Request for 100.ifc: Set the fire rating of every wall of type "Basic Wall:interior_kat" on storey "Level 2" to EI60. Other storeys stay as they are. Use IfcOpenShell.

First a look at what the model holds.

```python
import ifcopenshell
import ifcopenshell.util.element

model = ifcopenshell.open("100.ifc")
print(model.schema)
storey = next(s for s in model.by_type("IfcBuildingStorey") if s.Name == "Level 2")
walls = [e for e in ifcopenshell.util.element.get_decomposition(storey) if e.is_a("IfcWall")]
seen = {}
for e in walls:
    element_type = ifcopenshell.util.element.get_type(e)
    key = (element_type.Name if element_type != e and element_type else None, ifcopenshell.util.element.get_pset(e, "Pset_WallCommon", "FireRating"))
    seen[key] = seen.get(key, 0) + 1
for (name, value), count in sorted(seen.items(), key=str):
    print(count, "x", name, "|", value)
```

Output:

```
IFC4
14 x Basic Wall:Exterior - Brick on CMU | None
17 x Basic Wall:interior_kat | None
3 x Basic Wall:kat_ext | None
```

```python
import ifcopenshell
import ifcopenshell.api.pset
import ifcopenshell.util.element

model = ifcopenshell.open("100.ifc")

storey = next(s for s in model.by_type("IfcBuildingStorey") if s.Name == "Level 2")
walls = [e for e in ifcopenshell.util.element.get_decomposition(storey) if e.is_a("IfcWall")]

count = 0
for e in walls:
    element_type = ifcopenshell.util.element.get_type(e)
    if element_type in (None, e) or element_type.Name != "Basic Wall:interior_kat":
        continue
    # add_pset returns the element's existing set when there is one.
    pset = ifcopenshell.api.pset.add_pset(model, product=e, name="Pset_WallCommon")
    ifcopenshell.api.pset.edit_pset(model, pset=pset, properties={"FireRating": "EI60"})
    count += 1

print(count, "walls updated")

model.write("100_edited.ifc")
```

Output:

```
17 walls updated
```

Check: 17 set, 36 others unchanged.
